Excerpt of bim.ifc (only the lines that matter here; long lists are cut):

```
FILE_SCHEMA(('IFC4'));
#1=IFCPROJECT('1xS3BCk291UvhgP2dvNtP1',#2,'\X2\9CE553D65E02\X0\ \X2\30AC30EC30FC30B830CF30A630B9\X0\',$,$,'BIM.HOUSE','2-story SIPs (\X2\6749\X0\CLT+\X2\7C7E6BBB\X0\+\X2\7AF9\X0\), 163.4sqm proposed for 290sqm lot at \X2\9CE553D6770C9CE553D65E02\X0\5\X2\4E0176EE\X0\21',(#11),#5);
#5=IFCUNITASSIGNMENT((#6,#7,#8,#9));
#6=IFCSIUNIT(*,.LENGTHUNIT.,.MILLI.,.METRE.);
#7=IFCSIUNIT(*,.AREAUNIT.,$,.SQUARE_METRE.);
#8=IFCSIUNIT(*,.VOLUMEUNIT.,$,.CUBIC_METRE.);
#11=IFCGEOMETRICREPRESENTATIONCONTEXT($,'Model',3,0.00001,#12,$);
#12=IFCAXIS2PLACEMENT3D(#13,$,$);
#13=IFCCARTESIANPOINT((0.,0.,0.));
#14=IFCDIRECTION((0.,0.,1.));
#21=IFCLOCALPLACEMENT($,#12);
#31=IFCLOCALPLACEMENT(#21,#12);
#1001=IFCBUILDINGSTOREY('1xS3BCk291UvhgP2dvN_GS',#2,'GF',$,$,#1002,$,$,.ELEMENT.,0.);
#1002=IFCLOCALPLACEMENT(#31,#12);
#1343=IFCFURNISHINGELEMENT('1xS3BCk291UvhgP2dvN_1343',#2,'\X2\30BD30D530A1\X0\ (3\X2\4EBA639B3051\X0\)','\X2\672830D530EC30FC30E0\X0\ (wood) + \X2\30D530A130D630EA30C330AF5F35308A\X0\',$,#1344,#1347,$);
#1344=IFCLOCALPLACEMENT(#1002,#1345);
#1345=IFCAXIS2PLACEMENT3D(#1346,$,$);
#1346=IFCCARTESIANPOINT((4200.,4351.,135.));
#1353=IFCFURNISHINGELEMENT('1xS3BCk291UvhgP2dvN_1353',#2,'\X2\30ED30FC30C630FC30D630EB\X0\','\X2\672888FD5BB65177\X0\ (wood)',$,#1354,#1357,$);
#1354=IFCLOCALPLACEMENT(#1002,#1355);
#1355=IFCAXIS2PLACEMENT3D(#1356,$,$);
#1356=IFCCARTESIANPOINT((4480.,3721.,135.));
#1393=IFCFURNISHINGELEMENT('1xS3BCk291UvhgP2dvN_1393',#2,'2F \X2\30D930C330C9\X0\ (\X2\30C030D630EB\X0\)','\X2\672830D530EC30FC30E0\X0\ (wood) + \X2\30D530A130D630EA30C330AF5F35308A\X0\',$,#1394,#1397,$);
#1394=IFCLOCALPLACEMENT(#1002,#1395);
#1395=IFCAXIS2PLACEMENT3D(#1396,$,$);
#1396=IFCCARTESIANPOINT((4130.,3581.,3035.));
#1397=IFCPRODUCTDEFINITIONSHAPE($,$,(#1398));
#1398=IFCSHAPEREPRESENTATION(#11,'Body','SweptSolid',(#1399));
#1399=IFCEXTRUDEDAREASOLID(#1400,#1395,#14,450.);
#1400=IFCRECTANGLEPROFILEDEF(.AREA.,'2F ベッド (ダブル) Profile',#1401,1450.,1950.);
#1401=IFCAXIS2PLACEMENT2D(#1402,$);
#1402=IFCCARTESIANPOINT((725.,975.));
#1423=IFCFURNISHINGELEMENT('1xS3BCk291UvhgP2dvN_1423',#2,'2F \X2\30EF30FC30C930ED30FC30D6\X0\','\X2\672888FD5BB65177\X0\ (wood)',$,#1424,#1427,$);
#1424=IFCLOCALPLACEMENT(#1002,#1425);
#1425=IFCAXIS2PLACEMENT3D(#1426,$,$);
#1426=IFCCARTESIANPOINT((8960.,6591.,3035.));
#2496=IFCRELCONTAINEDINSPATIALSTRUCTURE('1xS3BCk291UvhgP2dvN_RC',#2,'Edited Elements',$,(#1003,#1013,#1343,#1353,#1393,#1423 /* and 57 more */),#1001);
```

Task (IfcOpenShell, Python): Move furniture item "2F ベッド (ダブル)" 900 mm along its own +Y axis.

```python
import ifcopenshell
import ifcopenshell.api.geometry
import ifcopenshell.util.placement
import ifcopenshell.util.unit

model = ifcopenshell.open("bim.ifc")
unit_scale = ifcopenshell.util.unit.calculate_unit_scale(model)

item = model.by_guid("1xS3BCk291UvhgP2dvN_1393")
matrix = ifcopenshell.util.placement.get_local_placement(item.ObjectPlacement)
matrix[:3, 3] += matrix[:3, 1] * 0.9 / unit_scale
ifcopenshell.api.geometry.edit_object_placement(model, product=item, matrix=matrix, is_si=False)

print(ifcopenshell.util.placement.get_local_placement(item.ObjectPlacement).round(3) + 0.0)

model.write("bim_rev.ifc")
```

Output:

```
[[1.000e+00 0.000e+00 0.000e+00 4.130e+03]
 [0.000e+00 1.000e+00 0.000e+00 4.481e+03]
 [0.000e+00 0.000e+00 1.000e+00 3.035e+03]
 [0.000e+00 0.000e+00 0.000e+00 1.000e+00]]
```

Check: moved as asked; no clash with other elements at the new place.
